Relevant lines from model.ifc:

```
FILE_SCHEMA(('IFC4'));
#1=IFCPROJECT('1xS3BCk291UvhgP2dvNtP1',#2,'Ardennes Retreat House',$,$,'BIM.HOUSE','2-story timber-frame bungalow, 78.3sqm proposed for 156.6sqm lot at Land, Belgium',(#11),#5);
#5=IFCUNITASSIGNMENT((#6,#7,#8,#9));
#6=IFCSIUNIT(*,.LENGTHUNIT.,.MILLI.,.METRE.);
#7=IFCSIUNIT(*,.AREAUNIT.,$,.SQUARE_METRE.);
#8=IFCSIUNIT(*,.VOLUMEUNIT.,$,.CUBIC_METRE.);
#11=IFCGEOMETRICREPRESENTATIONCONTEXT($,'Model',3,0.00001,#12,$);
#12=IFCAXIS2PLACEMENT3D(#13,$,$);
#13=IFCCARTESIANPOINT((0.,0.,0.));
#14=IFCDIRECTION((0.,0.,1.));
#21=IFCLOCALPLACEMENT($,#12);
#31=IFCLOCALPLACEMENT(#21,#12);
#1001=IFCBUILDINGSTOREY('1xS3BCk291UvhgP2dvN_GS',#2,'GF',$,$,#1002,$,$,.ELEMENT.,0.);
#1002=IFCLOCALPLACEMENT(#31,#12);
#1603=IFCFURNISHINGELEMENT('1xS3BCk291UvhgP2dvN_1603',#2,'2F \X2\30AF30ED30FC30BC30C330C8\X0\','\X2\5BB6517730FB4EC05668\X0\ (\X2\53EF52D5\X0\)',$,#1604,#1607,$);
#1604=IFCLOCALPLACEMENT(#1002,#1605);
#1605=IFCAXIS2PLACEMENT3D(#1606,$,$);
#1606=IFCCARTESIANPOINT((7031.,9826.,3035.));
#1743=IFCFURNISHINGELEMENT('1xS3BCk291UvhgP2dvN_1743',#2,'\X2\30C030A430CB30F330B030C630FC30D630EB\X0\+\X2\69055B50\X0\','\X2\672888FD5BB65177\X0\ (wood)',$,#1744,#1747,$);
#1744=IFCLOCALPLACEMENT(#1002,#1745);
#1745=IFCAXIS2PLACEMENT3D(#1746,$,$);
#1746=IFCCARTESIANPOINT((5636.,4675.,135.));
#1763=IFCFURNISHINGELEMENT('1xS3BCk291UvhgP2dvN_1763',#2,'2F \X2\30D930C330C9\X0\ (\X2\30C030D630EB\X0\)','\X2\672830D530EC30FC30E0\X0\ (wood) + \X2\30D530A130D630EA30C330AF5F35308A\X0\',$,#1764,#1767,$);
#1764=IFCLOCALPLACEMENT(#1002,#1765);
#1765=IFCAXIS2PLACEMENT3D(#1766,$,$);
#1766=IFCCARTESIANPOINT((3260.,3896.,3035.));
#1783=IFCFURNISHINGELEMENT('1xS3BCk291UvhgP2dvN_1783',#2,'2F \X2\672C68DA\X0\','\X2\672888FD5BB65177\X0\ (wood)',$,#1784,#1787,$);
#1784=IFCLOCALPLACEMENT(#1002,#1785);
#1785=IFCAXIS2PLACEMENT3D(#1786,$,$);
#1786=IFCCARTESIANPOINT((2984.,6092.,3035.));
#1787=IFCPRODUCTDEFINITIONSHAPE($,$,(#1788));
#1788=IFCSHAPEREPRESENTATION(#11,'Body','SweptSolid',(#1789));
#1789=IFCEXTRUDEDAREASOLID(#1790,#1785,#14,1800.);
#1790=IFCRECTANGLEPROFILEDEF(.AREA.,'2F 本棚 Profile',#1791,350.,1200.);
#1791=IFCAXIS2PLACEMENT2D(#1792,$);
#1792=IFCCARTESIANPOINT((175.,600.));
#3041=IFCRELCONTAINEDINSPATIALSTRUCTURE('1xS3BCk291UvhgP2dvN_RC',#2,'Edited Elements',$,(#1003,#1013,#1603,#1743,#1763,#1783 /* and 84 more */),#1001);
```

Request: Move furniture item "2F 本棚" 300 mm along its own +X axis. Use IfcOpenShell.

```python
import ifcopenshell
import ifcopenshell.api.geometry
import ifcopenshell.util.placement
import ifcopenshell.util.unit

model = ifcopenshell.open("model.ifc")
unit_scale = ifcopenshell.util.unit.calculate_unit_scale(model)

item = model.by_id(1783)
matrix = ifcopenshell.util.placement.get_local_placement(item.ObjectPlacement)
matrix[:3, 3] += matrix[:3, 0] * 0.3 / unit_scale
ifcopenshell.api.geometry.edit_object_placement(model, product=item, matrix=matrix, is_si=False)

print(ifcopenshell.util.placement.get_local_placement(item.ObjectPlacement).round(3) + 0.0)

model.write("model-out.ifc")
```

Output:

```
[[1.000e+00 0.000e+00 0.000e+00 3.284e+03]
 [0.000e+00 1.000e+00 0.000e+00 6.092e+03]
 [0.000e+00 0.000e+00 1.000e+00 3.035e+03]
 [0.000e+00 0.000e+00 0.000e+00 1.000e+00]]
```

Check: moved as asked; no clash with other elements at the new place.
